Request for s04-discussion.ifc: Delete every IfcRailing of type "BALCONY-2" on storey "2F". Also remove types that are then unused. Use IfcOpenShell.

First a look at what the model holds.

```python
import ifcopenshell
import ifcopenshell.util.element

model = ifcopenshell.open("s04-discussion.ifc")
print(model.schema)
storey = next(s for s in model.by_type("IfcBuildingStorey") if s.Name == "2F")
railings = [e for e in ifcopenshell.util.element.get_decomposition(storey) if e.is_a("IfcRailing")]
seen = {}
for e in railings:
    element_type = ifcopenshell.util.element.get_type(e)
    name = element_type.Name if element_type not in (None, e) else None
    seen[name] = seen.get(name, 0) + 1
for name, count in sorted(seen.items(), key=str):
    print(count, "x", name)
```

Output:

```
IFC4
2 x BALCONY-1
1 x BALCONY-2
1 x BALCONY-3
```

```python
import ifcopenshell
import ifcopenshell.api.root
import ifcopenshell.util.element

model = ifcopenshell.open("s04-discussion.ifc")

storey = next(s for s in model.by_type("IfcBuildingStorey") if s.Name == "2F")
railings = [e for e in ifcopenshell.util.element.get_decomposition(storey) if e.is_a("IfcRailing")]
targets = [e for e in railings if (t := ifcopenshell.util.element.get_type(e)) not in (None, e) and t.Name == "BALCONY-2"]
types = {ifcopenshell.util.element.get_type(e) for e in targets} - {None, *targets}

for e in targets:
    ifcopenshell.api.root.remove_product(model, product=e)
print(len(targets), "removed")

unused = [t for t in types if not ifcopenshell.util.element.get_types(t)]
for t in unused:
    ifcopenshell.api.root.remove_product(model, product=t)
print(len(unused), "unused types removed")

model.write("s04-discussion_v2.ifc")
```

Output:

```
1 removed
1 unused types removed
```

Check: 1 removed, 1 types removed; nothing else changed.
